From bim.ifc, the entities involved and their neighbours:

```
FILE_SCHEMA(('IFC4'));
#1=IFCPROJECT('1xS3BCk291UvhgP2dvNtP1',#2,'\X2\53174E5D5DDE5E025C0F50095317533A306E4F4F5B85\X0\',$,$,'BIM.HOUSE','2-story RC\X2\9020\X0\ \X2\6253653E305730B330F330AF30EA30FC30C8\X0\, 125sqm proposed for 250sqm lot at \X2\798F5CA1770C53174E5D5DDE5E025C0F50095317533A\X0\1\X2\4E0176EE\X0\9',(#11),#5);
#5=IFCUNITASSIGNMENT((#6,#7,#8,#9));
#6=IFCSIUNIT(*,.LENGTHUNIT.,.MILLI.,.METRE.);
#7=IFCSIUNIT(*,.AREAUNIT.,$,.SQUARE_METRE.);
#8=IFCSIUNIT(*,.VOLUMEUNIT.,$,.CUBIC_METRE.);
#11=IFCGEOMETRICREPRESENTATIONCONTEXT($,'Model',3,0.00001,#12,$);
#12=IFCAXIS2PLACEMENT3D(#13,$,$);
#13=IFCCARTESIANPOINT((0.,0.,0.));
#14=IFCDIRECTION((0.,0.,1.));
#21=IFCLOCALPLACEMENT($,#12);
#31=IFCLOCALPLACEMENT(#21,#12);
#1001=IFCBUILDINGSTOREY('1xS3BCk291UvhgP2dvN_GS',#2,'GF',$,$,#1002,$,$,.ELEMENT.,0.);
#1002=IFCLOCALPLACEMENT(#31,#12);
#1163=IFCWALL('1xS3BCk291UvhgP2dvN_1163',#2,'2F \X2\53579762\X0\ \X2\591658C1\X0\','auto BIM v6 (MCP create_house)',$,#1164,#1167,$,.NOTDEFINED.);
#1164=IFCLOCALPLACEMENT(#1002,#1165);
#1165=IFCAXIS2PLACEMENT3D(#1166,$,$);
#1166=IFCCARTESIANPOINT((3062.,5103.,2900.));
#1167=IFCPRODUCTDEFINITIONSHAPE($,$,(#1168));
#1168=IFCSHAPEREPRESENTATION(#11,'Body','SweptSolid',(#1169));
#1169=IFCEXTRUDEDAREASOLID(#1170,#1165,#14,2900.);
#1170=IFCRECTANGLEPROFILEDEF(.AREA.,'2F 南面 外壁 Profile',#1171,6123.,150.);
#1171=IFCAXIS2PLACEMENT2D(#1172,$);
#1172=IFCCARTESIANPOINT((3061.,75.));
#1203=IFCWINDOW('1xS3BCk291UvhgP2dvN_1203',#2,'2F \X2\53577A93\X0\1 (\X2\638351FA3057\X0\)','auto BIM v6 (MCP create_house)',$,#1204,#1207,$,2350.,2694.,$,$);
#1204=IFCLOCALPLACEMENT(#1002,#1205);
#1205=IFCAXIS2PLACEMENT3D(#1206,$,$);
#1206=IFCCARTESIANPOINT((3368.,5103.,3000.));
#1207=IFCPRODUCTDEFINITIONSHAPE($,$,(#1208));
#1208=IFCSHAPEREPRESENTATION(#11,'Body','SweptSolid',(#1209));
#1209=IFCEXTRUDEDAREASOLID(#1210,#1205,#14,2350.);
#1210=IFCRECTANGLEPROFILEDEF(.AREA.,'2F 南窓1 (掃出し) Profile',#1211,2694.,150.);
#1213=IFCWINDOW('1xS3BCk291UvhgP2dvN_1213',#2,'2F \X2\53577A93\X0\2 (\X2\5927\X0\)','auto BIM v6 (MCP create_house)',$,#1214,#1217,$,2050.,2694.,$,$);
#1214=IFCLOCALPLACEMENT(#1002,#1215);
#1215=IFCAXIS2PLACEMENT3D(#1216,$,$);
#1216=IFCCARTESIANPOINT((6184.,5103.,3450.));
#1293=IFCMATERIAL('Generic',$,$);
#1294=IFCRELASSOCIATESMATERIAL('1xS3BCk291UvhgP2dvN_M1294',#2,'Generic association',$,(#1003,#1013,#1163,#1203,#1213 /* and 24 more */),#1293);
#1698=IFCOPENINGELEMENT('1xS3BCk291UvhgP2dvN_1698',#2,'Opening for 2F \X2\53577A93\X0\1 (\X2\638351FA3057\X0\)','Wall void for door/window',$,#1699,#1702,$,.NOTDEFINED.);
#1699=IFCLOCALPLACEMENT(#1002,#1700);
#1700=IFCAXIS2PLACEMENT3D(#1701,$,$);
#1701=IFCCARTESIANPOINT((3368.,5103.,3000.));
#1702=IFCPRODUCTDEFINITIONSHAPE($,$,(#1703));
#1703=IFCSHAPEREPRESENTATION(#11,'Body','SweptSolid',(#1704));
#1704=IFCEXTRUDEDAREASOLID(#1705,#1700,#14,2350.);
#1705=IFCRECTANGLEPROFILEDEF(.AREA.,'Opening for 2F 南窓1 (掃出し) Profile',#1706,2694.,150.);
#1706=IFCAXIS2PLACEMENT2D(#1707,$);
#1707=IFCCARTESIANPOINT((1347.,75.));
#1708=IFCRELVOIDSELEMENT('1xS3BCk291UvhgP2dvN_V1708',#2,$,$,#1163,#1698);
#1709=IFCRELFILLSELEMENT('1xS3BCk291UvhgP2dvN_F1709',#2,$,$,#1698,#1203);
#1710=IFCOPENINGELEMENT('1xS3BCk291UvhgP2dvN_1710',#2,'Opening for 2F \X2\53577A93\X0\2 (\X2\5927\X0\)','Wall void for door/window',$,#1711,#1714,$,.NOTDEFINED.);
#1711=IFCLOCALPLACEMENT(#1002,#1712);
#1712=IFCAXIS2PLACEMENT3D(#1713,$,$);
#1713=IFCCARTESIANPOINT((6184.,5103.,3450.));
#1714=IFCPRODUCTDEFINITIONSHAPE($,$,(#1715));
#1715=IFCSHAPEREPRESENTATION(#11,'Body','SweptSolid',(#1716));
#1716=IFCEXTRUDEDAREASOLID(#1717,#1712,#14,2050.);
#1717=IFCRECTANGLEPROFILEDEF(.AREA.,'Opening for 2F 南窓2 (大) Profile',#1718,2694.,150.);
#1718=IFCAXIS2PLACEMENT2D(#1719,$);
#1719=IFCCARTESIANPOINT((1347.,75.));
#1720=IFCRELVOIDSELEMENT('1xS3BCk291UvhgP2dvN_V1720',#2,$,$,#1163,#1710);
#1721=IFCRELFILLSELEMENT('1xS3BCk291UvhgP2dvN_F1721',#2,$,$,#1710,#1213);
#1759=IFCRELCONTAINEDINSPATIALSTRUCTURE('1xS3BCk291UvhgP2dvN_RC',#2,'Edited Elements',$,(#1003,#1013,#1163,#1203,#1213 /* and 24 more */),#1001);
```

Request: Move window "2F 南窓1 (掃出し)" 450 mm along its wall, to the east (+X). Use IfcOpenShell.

```python
import ifcopenshell
import ifcopenshell.api.geometry
import ifcopenshell.util.placement
import ifcopenshell.util.unit

model = ifcopenshell.open("bim.ifc")
unit_scale = ifcopenshell.util.unit.calculate_unit_scale(model)

window = model.by_guid("1xS3BCk291UvhgP2dvN_1203")
opening = window.FillsVoids[0].RelatingOpeningElement
wall = opening.VoidsElements[0].RelatingBuildingElement

wall_matrix = ifcopenshell.util.placement.get_local_placement(wall.ObjectPlacement)
shift = wall_matrix[:3, 0] * 0.45 / unit_scale
before = ifcopenshell.util.placement.get_local_placement(window.ObjectPlacement)[:3, 3].copy()

# The window is not placed relative to its opening, so move both.
for product in (opening, window):
    matrix = ifcopenshell.util.placement.get_local_placement(product.ObjectPlacement)
    matrix[:3, 3] += shift
    ifcopenshell.api.geometry.edit_object_placement(model, product=product, matrix=matrix, is_si=False)

after = ifcopenshell.util.placement.get_local_placement(window.ObjectPlacement)[:3, 3]
print("window moved by", (after - before).round(3) + 0.0)

model.write("bim_edited.ifc")
```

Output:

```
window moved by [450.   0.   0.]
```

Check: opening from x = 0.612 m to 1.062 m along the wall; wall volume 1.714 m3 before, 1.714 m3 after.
